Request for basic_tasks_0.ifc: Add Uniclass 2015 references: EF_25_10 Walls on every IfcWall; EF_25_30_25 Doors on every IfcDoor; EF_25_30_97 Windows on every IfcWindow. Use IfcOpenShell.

First a look at what the model holds.

```python
import ifcopenshell

model = ifcopenshell.open("basic_tasks_0.ifc")
print(model.schema)
print("classifications:", [c.Name for c in model.by_type("IfcClassification")])
for ifc_class in ("IfcDoor", "IfcRoof", "IfcStair", "IfcWall", "IfcWindow"):
    print(ifc_class, len(model.by_type(ifc_class)))
```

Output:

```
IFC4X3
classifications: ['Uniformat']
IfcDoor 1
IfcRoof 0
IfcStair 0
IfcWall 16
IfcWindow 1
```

```python
import ifcopenshell
import ifcopenshell.api.classification

model = ifcopenshell.open("basic_tasks_0.ifc")

system = ifcopenshell.api.classification.add_classification(model, classification="Uniclass 2015")

codes = {
    "IfcWall": ("EF_25_10", "Walls"),
    "IfcDoor": ("EF_25_30_25", "Doors"),
    "IfcWindow": ("EF_25_30_97", "Windows"),
}
for ifc_class, (code, name) in codes.items():
    products = model.by_type(ifc_class)
    ifcopenshell.api.classification.add_reference(
        model, products=products, classification=system, identification=code, name=name
    )
    print(code, len(products))

model.write("basic_tasks_0_v2.ifc")
```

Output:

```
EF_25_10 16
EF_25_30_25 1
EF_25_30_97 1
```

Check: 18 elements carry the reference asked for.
